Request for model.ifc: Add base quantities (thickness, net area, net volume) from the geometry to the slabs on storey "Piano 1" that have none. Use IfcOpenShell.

First a look at what the model holds.

```python
import ifcopenshell
import ifcopenshell.util.element
import ifcopenshell.util.unit

model = ifcopenshell.open("model.ifc")
print(model.schema)
for unit_type in ("LENGTHUNIT", "AREAUNIT", "VOLUMEUNIT"):
    print(unit_type, ifcopenshell.util.unit.calculate_unit_scale(model, unit_type))
storey = next(s for s in model.by_type("IfcBuildingStorey") if s.Name == "Piano 1")
slabs = [e for e in ifcopenshell.util.element.get_decomposition(storey) if e.is_a("IfcSlab")]
for e in sorted(slabs, key=lambda e: e.id()):
    print(e.id(), e.is_a(), e.Name, list(ifcopenshell.util.element.get_psets(e, qtos_only=True)), sep=" | ")
```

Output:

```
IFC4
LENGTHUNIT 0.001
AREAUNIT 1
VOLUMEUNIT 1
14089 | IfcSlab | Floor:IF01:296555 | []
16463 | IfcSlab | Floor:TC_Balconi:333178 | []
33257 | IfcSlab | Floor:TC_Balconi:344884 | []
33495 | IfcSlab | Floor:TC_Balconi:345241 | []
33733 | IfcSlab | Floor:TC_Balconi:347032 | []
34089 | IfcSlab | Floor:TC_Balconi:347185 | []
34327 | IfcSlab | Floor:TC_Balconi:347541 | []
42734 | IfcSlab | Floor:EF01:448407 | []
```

```python
import ifcopenshell
import ifcopenshell.api.pset
import ifcopenshell.geom
import ifcopenshell.util.element
import ifcopenshell.util.shape
import ifcopenshell.util.unit

model = ifcopenshell.open("model.ifc")
unit_scale = ifcopenshell.util.unit.calculate_unit_scale(model)
area_scale = ifcopenshell.util.unit.calculate_unit_scale(model, "AREAUNIT")
volume_scale = ifcopenshell.util.unit.calculate_unit_scale(model, "VOLUMEUNIT")
settings = ifcopenshell.geom.settings()

storey = next(s for s in model.by_type("IfcBuildingStorey") if s.Name == "Piano 1")
slabs = [e for e in ifcopenshell.util.element.get_decomposition(storey) if e.is_a("IfcSlab")]

for e in sorted(slabs, key=lambda e: e.id()):
    if ifcopenshell.util.element.get_psets(e, qtos_only=True, should_inherit=False):
        continue
    # Geometry comes back in metres, in the element's own axes.
    shape = ifcopenshell.geom.create_shape(settings, e)
    values = {
        "Width": ifcopenshell.util.shape.get_z(shape.geometry) / unit_scale,
        "NetArea": ifcopenshell.util.shape.get_footprint_area(shape.geometry) / area_scale,
        "NetVolume": ifcopenshell.util.shape.get_volume(shape.geometry) / volume_scale,
    }
    qto = ifcopenshell.api.pset.add_qto(model, product=e, name="Qto_SlabBaseQuantities")
    ifcopenshell.api.pset.edit_qto(model, qto=qto, properties=values)
    print(e.id(), {k: round(v, 3) for k, v in values.items()})

model.write("model-out.ifc")
```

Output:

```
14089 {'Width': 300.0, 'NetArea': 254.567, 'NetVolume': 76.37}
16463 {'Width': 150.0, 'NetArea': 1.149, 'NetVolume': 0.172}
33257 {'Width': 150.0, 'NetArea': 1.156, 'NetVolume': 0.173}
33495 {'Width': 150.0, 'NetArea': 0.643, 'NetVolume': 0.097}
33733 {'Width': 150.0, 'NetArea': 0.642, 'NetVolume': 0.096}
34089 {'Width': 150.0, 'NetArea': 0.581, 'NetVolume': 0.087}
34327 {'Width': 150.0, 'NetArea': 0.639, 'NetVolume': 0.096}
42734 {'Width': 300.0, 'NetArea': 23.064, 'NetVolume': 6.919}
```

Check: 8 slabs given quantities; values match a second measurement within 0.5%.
